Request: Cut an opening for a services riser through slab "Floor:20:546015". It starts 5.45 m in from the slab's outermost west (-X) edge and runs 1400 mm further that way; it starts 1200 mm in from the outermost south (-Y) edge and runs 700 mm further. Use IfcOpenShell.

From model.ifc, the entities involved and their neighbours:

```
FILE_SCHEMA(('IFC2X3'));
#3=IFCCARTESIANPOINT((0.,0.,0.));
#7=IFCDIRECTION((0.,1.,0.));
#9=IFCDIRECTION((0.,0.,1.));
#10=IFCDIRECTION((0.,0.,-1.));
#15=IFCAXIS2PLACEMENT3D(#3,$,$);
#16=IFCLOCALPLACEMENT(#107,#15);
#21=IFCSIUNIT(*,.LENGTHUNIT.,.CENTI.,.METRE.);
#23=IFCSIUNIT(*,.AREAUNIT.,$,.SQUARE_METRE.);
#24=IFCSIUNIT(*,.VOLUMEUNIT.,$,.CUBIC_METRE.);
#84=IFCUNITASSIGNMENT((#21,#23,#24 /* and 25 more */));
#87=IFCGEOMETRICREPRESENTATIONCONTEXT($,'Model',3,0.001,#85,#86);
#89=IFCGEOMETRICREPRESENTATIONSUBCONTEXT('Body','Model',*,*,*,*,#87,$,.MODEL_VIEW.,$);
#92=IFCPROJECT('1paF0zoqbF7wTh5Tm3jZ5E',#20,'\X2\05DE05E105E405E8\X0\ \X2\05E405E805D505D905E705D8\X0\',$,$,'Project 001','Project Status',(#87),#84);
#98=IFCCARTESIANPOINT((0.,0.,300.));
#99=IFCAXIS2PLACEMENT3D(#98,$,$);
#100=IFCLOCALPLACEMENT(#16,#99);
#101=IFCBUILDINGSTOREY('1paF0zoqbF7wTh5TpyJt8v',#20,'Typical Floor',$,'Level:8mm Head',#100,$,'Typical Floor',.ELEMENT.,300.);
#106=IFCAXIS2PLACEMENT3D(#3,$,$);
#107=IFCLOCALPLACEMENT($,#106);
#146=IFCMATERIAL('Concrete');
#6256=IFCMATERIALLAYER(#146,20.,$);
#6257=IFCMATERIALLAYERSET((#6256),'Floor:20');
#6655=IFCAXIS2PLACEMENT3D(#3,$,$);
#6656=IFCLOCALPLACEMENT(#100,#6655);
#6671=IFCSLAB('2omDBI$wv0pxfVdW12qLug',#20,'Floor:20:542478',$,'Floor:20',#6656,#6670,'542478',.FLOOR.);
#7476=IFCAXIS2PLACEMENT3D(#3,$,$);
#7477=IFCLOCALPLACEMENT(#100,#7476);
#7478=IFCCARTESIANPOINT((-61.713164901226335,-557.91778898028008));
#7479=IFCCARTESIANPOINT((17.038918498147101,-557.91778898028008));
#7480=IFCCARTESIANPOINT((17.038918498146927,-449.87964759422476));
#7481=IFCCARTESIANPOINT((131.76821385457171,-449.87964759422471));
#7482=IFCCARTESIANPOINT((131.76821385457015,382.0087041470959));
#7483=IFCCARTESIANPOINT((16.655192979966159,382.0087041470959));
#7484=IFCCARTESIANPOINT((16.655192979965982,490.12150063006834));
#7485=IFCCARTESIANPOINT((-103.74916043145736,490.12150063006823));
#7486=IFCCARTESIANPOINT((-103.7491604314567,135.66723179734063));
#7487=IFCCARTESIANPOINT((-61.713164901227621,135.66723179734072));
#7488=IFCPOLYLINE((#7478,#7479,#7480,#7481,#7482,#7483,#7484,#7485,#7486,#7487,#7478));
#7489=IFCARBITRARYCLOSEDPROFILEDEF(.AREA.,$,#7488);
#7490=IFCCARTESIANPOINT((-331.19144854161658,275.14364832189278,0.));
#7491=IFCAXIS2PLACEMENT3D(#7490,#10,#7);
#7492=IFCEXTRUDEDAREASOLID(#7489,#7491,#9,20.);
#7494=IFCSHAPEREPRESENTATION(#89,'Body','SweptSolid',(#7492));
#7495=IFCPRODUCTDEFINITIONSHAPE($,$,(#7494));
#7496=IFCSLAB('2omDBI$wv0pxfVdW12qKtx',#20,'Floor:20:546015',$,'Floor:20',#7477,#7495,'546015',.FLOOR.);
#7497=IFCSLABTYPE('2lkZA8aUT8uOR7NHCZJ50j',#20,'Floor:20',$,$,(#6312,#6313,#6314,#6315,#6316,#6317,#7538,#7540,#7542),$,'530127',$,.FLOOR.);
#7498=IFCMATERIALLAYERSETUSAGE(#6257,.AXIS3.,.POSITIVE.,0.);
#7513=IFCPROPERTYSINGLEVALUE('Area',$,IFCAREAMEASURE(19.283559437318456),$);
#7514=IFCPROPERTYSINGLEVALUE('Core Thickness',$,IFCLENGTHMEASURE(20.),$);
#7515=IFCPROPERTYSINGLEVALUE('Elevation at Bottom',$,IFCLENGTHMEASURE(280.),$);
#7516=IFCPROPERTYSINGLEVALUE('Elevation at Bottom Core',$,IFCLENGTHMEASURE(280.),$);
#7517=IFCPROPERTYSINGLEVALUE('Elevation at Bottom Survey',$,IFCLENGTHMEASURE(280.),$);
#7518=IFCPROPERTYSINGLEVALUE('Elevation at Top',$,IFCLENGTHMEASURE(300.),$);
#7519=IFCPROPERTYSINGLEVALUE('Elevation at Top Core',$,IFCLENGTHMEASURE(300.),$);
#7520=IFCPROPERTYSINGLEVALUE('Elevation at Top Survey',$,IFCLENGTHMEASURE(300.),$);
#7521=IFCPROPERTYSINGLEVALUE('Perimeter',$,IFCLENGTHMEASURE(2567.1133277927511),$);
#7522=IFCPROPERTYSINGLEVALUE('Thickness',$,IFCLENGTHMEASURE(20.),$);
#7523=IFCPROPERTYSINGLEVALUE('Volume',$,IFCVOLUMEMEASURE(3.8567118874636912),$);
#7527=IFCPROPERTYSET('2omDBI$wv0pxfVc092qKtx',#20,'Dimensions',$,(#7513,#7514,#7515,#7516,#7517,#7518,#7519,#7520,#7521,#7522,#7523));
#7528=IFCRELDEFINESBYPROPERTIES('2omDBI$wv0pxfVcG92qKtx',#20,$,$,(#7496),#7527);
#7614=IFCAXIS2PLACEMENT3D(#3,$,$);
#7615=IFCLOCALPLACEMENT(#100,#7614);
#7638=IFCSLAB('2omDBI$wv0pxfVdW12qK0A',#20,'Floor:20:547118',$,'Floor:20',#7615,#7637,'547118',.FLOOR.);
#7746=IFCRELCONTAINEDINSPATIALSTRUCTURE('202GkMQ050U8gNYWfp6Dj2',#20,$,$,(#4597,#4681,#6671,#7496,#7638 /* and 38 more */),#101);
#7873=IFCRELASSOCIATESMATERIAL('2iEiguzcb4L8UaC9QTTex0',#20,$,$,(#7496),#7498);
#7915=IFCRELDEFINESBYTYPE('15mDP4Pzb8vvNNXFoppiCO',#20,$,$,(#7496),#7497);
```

```python
import numpy as np
import ifcopenshell
import ifcopenshell.api.feature
import ifcopenshell.api.geometry
import ifcopenshell.api.pset
import ifcopenshell.api.root
import ifcopenshell.geom
import ifcopenshell.util.element
import ifcopenshell.util.placement
import ifcopenshell.util.representation
import ifcopenshell.util.shape
import ifcopenshell.util.unit

model = ifcopenshell.open("model.ifc")
unit_scale = ifcopenshell.util.unit.calculate_unit_scale(model)
area_scale = ifcopenshell.util.unit.calculate_unit_scale(model, "AREAUNIT")
volume_scale = ifcopenshell.util.unit.calculate_unit_scale(model, "VOLUMEUNIT")
settings = ifcopenshell.geom.settings()


def volume(element):
    """Net volume in cubic metres, openings subtracted."""
    shape = ifcopenshell.geom.create_shape(settings, element)
    return ifcopenshell.util.shape.get_volume(shape.geometry)


slab = model.by_id(7496)
before = volume(slab)

# Extent in the slab's own axes, in metres. The edges named are its -X and -Y sides.
slab_shape = ifcopenshell.geom.create_shape(settings, slab)
vertices = ifcopenshell.util.shape.get_vertices(slab_shape.geometry)
x_min, y_min, bottom = vertices.min(axis=0)
top = vertices[:, 2].max()

opening = ifcopenshell.api.root.create_entity(model, ifc_class="IfcOpeningElement", name="Services riser opening")
context = ifcopenshell.util.representation.get_context(model, "Model", "Body", "MODEL_VIEW")
width, depth = 1.4, 0.7
outline = [(0.0, 0.0), (width, 0.0), (width, depth), (0.0, depth), (0.0, 0.0)]
# Overshoot both faces by 50 mm so the cut is clean.
shape = ifcopenshell.api.geometry.add_slab_representation(
    model, context=context, depth=top - bottom + 0.1, polyline=outline
)
ifcopenshell.api.geometry.assign_representation(model, product=opening, representation=shape)

matrix = ifcopenshell.util.placement.get_local_placement(slab.ObjectPlacement)
matrix[:, 3] = matrix @ np.append(np.array([x_min + 5.45, y_min + 1.2, bottom - 0.05]) / unit_scale, 1.0)
ifcopenshell.api.geometry.edit_object_placement(model, product=opening, matrix=matrix, is_si=False)
ifcopenshell.api.feature.add_feature(model, feature=opening, element=slab)

after = volume(slab)

# Update the slab's stored quantities.
pset = model.by_id(ifcopenshell.util.element.get_pset(slab, "Dimensions", should_inherit=False)["id"])
ifcopenshell.api.pset.edit_pset(model, pset=pset, properties={
    "Area": model.create_entity("IfcAreaMeasure", after / (top - bottom) / area_scale),
    "Volume": model.create_entity("IfcVolumeMeasure", after / volume_scale),
})

print(f"slab volume {before:.3f} -> {after:.3f} m3")

model.write("model_v2.ifc")
```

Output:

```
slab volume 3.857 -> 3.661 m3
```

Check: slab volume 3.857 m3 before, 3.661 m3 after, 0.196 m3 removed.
